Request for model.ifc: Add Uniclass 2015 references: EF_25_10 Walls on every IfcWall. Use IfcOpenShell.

First a look at what the model holds.

```python
import ifcopenshell

model = ifcopenshell.open("model.ifc")
print(model.schema)
print("classifications:", [c.Name for c in model.by_type("IfcClassification")])
for ifc_class in ("IfcDoor", "IfcRoof", "IfcStair", "IfcWall", "IfcWindow"):
    print(ifc_class, len(model.by_type(ifc_class)))
```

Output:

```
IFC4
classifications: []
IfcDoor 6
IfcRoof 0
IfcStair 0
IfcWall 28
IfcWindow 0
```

```python
import ifcopenshell
import ifcopenshell.api.classification

model = ifcopenshell.open("model.ifc")

system = ifcopenshell.api.classification.add_classification(model, classification="Uniclass 2015")

codes = {
    "IfcWall": ("EF_25_10", "Walls"),
}
for ifc_class, (code, name) in codes.items():
    products = model.by_type(ifc_class)
    ifcopenshell.api.classification.add_reference(
        model, products=products, classification=system, identification=code, name=name
    )
    print(code, len(products))

model.write("model-out.ifc")
```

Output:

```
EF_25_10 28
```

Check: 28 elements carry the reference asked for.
